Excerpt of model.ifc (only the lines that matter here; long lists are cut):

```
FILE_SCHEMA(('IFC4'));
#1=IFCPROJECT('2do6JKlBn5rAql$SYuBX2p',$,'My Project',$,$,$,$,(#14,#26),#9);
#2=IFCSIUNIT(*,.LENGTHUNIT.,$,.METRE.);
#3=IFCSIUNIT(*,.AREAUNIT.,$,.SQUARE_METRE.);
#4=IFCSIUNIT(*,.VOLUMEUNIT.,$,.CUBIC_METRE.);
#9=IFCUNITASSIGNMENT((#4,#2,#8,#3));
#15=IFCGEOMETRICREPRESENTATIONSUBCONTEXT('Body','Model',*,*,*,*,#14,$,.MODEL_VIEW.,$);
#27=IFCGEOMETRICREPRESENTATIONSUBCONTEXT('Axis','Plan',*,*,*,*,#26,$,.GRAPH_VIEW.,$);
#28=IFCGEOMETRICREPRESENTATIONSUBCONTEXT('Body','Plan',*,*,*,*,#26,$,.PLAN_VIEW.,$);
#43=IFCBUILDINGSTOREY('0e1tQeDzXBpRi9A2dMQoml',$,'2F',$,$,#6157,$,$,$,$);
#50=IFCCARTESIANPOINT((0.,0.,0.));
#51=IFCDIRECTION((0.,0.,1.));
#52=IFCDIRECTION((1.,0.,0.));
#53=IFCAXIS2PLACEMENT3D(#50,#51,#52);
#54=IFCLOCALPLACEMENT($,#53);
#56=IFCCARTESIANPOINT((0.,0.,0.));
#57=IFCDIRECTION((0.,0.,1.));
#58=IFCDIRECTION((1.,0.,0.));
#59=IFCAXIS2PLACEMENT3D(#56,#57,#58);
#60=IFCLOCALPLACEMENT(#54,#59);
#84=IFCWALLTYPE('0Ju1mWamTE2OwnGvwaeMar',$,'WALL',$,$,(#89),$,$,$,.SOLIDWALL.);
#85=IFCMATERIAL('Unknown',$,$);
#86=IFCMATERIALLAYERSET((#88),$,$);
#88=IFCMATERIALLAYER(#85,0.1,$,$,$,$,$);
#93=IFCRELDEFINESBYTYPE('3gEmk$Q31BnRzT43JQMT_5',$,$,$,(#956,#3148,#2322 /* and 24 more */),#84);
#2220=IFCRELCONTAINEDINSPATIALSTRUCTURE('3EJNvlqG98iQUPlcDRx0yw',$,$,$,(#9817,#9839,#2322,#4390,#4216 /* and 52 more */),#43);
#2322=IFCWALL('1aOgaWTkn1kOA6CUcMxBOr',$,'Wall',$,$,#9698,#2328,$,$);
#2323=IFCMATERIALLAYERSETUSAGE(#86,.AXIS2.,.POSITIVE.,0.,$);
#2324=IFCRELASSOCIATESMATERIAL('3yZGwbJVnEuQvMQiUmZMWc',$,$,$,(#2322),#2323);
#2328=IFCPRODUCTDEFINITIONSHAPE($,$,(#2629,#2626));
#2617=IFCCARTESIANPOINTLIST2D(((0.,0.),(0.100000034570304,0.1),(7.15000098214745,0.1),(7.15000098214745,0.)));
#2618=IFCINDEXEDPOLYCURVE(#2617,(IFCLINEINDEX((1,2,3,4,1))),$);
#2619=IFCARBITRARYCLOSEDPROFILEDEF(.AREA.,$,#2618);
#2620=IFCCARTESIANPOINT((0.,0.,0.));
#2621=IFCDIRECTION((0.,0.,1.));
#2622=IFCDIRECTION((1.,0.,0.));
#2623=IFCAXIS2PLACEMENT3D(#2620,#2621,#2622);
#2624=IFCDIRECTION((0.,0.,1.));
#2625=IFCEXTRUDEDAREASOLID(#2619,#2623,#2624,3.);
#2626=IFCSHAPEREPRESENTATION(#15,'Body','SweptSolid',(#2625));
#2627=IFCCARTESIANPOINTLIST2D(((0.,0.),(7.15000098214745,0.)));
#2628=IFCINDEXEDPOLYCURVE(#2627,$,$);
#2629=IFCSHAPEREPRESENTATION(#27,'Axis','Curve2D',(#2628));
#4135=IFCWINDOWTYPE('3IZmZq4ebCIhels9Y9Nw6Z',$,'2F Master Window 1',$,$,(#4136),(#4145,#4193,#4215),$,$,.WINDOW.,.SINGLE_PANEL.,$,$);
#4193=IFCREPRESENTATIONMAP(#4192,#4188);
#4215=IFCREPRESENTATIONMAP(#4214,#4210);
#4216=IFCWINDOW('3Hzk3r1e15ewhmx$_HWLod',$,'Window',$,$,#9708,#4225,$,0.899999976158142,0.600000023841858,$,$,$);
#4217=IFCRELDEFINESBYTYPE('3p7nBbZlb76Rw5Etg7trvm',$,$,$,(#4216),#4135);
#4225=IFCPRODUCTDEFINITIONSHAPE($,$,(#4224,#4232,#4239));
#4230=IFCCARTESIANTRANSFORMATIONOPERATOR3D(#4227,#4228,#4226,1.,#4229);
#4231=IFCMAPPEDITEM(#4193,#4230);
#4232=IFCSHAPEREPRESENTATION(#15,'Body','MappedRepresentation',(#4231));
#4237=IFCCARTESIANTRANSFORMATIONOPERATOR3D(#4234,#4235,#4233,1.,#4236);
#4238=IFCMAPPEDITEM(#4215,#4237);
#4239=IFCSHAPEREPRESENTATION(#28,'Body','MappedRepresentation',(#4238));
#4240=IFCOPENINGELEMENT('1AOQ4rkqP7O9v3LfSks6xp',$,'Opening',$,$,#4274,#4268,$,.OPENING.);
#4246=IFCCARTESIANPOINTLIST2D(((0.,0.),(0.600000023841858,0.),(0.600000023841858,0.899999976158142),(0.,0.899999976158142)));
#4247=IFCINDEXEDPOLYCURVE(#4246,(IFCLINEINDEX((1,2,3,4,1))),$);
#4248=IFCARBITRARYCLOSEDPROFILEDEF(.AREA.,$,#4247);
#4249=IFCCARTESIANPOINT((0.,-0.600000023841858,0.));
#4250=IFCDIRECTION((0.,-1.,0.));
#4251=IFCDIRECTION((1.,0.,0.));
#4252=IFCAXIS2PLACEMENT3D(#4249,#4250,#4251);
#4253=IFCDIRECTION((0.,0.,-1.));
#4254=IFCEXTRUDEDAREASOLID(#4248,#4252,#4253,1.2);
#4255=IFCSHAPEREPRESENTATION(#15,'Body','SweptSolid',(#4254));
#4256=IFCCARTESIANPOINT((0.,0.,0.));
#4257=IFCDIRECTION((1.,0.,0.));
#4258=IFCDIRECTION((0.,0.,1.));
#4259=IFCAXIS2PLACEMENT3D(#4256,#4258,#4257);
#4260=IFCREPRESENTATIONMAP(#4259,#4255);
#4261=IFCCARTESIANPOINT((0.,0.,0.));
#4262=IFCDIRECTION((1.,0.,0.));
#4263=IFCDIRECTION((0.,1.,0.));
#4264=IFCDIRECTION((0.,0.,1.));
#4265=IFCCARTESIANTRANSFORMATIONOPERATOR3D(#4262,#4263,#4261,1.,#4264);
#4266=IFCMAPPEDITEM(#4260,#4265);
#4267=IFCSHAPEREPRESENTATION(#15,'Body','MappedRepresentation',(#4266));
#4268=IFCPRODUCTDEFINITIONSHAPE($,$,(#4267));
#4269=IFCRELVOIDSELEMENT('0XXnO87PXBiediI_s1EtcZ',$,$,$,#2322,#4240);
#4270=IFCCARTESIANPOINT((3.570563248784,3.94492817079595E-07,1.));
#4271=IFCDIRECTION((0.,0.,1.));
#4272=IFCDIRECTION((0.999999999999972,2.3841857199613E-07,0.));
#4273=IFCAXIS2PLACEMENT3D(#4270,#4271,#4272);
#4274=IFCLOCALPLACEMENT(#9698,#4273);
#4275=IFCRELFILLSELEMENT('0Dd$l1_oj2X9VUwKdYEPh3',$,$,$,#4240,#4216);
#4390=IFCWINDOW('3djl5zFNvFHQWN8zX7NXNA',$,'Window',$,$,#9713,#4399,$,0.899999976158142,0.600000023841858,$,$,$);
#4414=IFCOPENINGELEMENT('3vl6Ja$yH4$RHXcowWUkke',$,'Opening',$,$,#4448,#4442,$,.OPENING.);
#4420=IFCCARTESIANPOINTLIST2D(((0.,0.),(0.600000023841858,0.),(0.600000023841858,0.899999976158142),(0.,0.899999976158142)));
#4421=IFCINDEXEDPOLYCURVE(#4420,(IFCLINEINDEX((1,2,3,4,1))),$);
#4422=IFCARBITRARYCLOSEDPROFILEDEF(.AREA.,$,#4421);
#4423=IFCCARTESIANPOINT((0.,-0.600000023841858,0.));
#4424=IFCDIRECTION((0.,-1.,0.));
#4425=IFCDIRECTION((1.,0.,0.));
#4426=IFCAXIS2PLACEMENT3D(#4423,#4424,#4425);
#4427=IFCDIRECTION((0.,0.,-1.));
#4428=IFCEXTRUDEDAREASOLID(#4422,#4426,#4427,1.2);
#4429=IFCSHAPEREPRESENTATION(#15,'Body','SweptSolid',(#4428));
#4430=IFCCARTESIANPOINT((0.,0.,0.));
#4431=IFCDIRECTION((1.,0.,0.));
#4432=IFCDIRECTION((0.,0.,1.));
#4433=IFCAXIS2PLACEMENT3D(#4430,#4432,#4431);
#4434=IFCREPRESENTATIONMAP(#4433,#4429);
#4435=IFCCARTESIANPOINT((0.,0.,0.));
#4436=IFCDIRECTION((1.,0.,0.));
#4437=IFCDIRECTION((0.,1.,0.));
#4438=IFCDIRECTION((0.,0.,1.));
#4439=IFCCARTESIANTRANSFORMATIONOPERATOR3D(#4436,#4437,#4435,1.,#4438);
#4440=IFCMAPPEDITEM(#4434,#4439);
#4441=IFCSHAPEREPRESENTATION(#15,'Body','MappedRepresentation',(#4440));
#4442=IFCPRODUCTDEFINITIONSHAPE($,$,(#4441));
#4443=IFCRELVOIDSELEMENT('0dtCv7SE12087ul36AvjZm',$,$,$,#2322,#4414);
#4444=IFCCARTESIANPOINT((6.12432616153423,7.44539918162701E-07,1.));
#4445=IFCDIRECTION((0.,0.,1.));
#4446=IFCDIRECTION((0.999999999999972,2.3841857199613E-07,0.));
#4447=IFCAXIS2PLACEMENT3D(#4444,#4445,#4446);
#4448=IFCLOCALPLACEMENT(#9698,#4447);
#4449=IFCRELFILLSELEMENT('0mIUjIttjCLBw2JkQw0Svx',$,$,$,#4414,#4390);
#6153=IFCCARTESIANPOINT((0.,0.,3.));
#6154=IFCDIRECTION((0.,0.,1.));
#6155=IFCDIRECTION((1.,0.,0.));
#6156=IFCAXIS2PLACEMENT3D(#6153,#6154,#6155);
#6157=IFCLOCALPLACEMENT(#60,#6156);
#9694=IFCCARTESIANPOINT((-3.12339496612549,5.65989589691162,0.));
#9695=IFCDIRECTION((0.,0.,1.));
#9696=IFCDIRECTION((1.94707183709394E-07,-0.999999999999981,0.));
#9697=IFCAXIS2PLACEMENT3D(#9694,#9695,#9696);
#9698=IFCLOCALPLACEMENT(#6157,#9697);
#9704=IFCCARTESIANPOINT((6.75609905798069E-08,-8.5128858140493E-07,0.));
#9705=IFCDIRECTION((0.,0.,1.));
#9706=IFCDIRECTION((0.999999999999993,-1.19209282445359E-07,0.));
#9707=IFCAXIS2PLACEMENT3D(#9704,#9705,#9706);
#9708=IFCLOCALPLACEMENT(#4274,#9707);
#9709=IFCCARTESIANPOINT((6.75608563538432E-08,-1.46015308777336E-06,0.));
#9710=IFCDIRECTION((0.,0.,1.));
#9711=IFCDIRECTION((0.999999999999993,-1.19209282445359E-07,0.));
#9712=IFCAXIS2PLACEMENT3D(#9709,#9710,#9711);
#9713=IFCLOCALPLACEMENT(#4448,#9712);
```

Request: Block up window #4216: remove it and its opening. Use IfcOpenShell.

```python
import ifcopenshell
import ifcopenshell.api.feature
import ifcopenshell.api.root
import ifcopenshell.geom
import ifcopenshell.util.shape

model = ifcopenshell.open("model.ifc")
settings = ifcopenshell.geom.settings()


def volume(element):
    """Net volume in cubic metres, openings subtracted."""
    shape = ifcopenshell.geom.create_shape(settings, element)
    return ifcopenshell.util.shape.get_volume(shape.geometry)


window = model.by_id(4216)
opening = window.FillsVoids[0].RelatingOpeningElement
wall = opening.VoidsElements[0].RelatingBuildingElement
before = volume(wall)

ifcopenshell.api.root.remove_product(model, product=window)
ifcopenshell.api.feature.remove_feature(model, feature=opening)

after = volume(wall)

print(f"wall volume {before:.3f} -> {after:.3f} m3")

model.write("model_rev.ifc")
```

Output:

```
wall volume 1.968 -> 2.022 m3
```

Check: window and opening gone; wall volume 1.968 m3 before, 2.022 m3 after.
